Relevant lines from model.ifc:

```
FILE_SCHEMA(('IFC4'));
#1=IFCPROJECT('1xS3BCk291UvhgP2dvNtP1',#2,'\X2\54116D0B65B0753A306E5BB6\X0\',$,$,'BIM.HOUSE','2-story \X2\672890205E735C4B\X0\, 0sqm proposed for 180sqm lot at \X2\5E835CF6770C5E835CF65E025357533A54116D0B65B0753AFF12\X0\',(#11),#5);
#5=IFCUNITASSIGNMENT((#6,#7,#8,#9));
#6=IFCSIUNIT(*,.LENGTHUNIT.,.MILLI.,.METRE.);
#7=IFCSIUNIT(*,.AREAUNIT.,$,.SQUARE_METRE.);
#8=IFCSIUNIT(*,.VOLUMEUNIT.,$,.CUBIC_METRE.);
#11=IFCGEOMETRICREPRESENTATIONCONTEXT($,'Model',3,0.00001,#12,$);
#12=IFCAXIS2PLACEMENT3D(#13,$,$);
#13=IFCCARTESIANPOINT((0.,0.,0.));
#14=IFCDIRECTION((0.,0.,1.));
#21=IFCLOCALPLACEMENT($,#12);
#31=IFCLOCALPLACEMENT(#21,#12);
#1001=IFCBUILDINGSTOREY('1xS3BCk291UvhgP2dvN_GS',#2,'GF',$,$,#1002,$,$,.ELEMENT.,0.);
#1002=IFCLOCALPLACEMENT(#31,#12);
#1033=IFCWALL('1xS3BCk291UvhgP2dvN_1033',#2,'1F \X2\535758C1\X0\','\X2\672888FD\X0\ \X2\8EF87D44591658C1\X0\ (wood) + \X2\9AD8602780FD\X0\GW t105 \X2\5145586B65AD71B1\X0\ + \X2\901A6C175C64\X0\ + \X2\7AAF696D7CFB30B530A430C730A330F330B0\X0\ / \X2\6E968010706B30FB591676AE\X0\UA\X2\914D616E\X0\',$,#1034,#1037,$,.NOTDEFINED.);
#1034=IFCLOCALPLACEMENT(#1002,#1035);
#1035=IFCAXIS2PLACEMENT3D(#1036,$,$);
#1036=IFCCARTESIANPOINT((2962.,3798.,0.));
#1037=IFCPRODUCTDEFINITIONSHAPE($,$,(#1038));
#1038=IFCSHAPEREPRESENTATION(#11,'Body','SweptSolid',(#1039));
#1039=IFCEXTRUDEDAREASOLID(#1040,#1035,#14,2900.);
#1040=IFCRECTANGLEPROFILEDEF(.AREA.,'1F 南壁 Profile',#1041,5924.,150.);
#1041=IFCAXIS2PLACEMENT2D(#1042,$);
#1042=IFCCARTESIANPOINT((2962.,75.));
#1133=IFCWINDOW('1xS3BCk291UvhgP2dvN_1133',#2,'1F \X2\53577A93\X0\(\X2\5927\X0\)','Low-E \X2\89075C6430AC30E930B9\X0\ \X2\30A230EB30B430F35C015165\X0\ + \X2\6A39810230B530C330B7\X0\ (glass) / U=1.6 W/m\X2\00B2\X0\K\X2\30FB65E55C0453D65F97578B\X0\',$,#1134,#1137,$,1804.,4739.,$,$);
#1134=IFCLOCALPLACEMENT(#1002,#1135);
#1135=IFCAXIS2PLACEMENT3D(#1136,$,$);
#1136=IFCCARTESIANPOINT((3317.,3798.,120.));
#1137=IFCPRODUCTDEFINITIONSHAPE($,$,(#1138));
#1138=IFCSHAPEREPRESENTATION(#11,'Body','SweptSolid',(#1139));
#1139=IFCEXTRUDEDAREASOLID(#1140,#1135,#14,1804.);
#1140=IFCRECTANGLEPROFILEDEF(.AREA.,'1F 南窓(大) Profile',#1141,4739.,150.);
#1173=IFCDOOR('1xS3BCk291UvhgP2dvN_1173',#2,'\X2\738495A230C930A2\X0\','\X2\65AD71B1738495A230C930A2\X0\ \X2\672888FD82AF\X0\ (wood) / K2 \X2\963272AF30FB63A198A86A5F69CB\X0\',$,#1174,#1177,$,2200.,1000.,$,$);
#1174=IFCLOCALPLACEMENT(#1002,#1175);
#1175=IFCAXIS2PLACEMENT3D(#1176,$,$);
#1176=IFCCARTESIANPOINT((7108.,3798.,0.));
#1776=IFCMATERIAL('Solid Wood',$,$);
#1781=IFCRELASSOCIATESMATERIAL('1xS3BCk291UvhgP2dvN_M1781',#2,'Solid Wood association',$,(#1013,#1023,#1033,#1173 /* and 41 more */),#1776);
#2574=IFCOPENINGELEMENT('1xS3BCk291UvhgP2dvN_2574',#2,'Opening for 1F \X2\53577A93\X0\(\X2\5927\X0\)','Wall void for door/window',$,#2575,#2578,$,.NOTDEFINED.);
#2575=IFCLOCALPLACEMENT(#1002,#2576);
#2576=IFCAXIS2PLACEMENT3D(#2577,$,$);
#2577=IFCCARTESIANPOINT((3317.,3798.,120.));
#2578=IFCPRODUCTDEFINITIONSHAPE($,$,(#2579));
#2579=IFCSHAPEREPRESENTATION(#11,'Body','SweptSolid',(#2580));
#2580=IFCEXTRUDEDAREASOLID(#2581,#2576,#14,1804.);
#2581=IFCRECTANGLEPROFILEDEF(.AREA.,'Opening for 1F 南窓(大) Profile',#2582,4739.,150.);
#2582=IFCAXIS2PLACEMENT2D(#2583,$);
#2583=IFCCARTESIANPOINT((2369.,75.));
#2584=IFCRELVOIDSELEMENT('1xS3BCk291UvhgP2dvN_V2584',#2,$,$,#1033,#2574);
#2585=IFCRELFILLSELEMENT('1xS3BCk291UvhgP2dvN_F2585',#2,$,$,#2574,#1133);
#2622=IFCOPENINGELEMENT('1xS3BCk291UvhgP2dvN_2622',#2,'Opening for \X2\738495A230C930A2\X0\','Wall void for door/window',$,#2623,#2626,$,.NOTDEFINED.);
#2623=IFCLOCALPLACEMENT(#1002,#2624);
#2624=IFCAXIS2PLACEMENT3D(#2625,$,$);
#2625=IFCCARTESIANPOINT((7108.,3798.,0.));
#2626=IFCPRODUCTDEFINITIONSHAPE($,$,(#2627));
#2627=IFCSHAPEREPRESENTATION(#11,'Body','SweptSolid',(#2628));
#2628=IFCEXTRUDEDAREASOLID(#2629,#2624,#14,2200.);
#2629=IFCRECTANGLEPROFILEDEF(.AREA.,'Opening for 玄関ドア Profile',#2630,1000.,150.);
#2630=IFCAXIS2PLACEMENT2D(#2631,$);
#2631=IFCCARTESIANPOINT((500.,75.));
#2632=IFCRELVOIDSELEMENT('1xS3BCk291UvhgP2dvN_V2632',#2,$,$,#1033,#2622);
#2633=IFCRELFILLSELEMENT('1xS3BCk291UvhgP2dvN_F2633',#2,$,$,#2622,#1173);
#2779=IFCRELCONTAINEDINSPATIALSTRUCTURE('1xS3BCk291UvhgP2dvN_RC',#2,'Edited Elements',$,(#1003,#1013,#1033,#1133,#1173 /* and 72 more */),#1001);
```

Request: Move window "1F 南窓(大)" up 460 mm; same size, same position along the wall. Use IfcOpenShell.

```python
import numpy as np
import ifcopenshell
import ifcopenshell.api.geometry
import ifcopenshell.util.placement
import ifcopenshell.util.unit

model = ifcopenshell.open("model.ifc")
unit_scale = ifcopenshell.util.unit.calculate_unit_scale(model)

window = model.by_id(1133)
opening = window.FillsVoids[0].RelatingOpeningElement
dz = 0.46 / unit_scale

shift = np.array([0.0, 0.0, dz])
# The window is not placed relative to its opening, so move both.
for product in (opening, window):
    matrix = ifcopenshell.util.placement.get_local_placement(product.ObjectPlacement)
    matrix[:3, 3] += shift
    ifcopenshell.api.geometry.edit_object_placement(model, product=product, matrix=matrix, is_si=False)

print(f"moved by {dz * unit_scale:+.3f} m")

model.write("model_updated.ifc")
```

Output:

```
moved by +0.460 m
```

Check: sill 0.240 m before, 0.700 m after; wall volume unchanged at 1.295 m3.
